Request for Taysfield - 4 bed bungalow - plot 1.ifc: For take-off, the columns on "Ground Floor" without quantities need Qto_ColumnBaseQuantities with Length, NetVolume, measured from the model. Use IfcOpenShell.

First a look at what the model holds.

```python
import ifcopenshell
import ifcopenshell.util.element
import ifcopenshell.util.unit

model = ifcopenshell.open("Taysfield - 4 bed bungalow - plot 1.ifc")
print(model.schema)
for unit_type in ("LENGTHUNIT", "AREAUNIT", "VOLUMEUNIT"):
    print(unit_type, ifcopenshell.util.unit.calculate_unit_scale(model, unit_type))
storey = next(s for s in model.by_type("IfcBuildingStorey") if s.Name == "Ground Floor")
columns = [e for e in ifcopenshell.util.element.get_decomposition(storey) if e.is_a("IfcColumn")]
for e in sorted(columns, key=lambda e: e.id()):
    print(e.id(), e.is_a(), e.Name, list(ifcopenshell.util.element.get_psets(e, qtos_only=True)), sep=" | ")
```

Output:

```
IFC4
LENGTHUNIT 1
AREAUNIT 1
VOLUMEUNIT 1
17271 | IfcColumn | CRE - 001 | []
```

```python
import ifcopenshell
import ifcopenshell.api.pset
import ifcopenshell.geom
import ifcopenshell.util.element
import ifcopenshell.util.shape
import ifcopenshell.util.unit

model = ifcopenshell.open("Taysfield - 4 bed bungalow - plot 1.ifc")
unit_scale = ifcopenshell.util.unit.calculate_unit_scale(model)
volume_scale = ifcopenshell.util.unit.calculate_unit_scale(model, "VOLUMEUNIT")
settings = ifcopenshell.geom.settings()

storey = next(s for s in model.by_type("IfcBuildingStorey") if s.Name == "Ground Floor")
columns = [e for e in ifcopenshell.util.element.get_decomposition(storey) if e.is_a("IfcColumn")]

for e in sorted(columns, key=lambda e: e.id()):
    if ifcopenshell.util.element.get_psets(e, qtos_only=True, should_inherit=False):
        continue
    # Geometry comes back in metres, in the element's own axes.
    shape = ifcopenshell.geom.create_shape(settings, e)
    values = {
        "Length": ifcopenshell.util.shape.get_z(shape.geometry) / unit_scale,
        "NetVolume": ifcopenshell.util.shape.get_volume(shape.geometry) / volume_scale,
    }
    qto = ifcopenshell.api.pset.add_qto(model, product=e, name="Qto_ColumnBaseQuantities")
    ifcopenshell.api.pset.edit_qto(model, qto=qto, properties=values)
    print(e.id(), {k: round(v, 3) for k, v in values.items()})

model.write("Taysfield - 4 bed bungalow - plot 1_v2.ifc")
```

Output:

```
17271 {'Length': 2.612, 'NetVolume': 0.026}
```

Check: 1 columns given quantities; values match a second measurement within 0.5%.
